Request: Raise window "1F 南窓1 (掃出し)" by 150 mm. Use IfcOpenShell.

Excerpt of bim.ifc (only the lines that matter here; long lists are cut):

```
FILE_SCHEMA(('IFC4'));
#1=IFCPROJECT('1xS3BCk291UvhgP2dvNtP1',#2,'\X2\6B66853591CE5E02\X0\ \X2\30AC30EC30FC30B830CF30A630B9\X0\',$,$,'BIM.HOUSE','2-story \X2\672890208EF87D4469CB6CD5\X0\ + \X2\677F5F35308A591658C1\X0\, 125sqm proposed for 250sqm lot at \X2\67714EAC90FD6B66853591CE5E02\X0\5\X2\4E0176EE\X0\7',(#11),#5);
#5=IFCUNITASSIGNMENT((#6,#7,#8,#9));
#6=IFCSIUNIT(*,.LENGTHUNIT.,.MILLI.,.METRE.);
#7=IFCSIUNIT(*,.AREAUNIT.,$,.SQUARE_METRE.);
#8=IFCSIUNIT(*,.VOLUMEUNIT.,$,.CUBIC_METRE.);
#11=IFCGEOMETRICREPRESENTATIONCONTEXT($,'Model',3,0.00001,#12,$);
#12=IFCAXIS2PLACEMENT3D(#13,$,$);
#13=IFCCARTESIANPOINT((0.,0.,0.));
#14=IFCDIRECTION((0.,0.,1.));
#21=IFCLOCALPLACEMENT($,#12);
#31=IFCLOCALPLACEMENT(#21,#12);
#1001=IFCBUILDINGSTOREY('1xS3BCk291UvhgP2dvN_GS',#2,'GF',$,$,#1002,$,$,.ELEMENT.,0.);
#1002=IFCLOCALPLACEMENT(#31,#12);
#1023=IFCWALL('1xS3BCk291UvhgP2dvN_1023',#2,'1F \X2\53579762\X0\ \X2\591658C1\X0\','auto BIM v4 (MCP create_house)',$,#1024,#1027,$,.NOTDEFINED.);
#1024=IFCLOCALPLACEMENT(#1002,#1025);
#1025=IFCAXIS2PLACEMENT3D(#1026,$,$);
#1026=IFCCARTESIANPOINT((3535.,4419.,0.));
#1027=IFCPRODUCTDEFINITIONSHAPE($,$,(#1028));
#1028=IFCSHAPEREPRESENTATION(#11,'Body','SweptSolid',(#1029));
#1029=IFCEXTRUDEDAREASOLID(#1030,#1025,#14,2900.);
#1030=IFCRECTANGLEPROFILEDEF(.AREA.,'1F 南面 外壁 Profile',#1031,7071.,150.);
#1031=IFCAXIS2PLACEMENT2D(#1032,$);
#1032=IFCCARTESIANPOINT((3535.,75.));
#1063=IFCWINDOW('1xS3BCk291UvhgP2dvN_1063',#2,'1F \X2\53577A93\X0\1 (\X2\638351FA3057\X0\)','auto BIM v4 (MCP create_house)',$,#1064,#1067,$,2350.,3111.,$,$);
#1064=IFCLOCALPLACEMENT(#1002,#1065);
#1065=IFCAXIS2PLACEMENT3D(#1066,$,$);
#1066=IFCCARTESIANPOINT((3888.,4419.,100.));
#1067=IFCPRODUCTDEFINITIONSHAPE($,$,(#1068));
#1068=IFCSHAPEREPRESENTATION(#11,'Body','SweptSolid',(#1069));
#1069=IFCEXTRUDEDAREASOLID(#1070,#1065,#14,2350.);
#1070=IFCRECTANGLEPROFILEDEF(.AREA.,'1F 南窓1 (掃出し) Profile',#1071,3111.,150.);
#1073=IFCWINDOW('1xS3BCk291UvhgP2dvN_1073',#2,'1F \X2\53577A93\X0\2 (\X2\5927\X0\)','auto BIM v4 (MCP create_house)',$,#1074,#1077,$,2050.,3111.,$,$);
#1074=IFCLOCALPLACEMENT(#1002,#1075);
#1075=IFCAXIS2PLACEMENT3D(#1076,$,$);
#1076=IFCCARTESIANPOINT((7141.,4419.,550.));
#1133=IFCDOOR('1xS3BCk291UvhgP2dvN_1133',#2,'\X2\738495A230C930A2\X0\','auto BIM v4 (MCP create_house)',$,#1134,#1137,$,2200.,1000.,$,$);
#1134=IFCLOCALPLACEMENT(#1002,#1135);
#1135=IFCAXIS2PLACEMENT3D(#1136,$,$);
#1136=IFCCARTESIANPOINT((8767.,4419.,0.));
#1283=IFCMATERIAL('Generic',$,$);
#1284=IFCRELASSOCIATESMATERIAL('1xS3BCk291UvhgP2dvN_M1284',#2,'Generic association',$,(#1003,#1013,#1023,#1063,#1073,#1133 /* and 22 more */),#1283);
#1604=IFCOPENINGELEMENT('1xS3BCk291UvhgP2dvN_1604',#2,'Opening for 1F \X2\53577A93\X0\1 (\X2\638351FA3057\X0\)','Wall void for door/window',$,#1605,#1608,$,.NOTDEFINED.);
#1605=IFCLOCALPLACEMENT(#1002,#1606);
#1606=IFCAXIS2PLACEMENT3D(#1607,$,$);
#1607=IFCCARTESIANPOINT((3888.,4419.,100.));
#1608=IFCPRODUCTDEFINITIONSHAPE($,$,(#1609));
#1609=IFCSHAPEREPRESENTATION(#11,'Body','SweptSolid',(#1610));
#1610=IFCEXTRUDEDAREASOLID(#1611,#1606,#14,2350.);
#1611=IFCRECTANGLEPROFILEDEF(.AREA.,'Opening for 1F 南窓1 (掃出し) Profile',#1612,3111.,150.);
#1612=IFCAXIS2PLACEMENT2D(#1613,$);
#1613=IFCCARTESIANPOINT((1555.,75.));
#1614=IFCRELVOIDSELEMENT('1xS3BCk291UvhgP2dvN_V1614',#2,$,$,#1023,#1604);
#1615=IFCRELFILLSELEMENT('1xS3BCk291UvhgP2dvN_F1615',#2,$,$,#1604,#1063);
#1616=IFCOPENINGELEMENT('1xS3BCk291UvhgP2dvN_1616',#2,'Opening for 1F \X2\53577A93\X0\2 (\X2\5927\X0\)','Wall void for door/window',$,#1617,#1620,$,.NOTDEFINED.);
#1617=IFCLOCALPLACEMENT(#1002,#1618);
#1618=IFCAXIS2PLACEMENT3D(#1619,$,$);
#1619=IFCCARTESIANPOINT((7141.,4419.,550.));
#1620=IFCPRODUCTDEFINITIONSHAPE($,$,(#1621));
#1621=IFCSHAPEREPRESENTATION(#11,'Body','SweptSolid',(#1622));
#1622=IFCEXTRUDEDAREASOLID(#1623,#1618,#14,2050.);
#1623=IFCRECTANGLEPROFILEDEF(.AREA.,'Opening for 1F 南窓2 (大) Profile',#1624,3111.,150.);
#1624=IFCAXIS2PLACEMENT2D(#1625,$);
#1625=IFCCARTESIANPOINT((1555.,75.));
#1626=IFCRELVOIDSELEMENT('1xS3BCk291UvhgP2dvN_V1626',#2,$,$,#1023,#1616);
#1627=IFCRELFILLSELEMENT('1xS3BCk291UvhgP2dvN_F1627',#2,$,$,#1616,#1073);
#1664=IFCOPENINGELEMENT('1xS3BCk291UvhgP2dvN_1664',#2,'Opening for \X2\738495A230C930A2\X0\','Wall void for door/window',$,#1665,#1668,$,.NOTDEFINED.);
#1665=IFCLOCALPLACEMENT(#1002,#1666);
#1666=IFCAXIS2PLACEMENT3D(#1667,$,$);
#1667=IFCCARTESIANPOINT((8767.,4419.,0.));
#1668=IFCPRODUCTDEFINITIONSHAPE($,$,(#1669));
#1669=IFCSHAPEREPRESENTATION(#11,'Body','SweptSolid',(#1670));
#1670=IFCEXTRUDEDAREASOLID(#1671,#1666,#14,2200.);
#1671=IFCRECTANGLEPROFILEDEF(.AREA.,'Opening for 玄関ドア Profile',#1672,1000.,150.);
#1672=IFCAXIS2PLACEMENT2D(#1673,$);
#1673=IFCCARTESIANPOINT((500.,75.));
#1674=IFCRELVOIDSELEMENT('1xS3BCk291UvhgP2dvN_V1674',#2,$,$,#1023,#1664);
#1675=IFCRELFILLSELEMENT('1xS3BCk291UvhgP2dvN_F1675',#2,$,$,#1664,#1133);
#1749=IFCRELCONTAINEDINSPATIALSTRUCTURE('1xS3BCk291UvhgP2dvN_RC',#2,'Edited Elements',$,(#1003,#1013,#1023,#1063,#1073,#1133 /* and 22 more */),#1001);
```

```python
import numpy as np
import ifcopenshell
import ifcopenshell.api.geometry
import ifcopenshell.util.placement
import ifcopenshell.util.unit

model = ifcopenshell.open("bim.ifc")
unit_scale = ifcopenshell.util.unit.calculate_unit_scale(model)

window = model.by_guid("1xS3BCk291UvhgP2dvN_1063")
opening = window.FillsVoids[0].RelatingOpeningElement
dz = 0.15 / unit_scale

shift = np.array([0.0, 0.0, dz])
# The window is not placed relative to its opening, so move both.
for product in (opening, window):
    matrix = ifcopenshell.util.placement.get_local_placement(product.ObjectPlacement)
    matrix[:3, 3] += shift
    ifcopenshell.api.geometry.edit_object_placement(model, product=product, matrix=matrix, is_si=False)

print(f"moved by {dz * unit_scale:+.3f} m")

model.write("bim-out.ifc")
```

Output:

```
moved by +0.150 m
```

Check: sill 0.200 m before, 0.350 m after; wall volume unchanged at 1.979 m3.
